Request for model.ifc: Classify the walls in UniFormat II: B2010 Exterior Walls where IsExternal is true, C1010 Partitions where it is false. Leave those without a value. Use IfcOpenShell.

First a look at what the model holds.

```python
import ifcopenshell
import ifcopenshell.util.element

model = ifcopenshell.open("model.ifc")
print(model.schema)
print("classifications:", [c.Name for c in model.by_type("IfcClassification")])
values = [ifcopenshell.util.element.get_pset(e, "Pset_WallCommon", "IsExternal") for e in model.by_type("IfcWall")]
for value in (True, False, None):
    print("IsExternal", value, values.count(value))
```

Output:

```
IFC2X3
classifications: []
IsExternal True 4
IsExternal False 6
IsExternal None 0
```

```python
import ifcopenshell
import ifcopenshell.api.classification
import ifcopenshell.util.element

model = ifcopenshell.open("model.ifc")

# IFC2X3 requires Source and Edition and has no link from the project to the system.
system = model.create_entity("IfcClassification", Source="ASTM", Edition="E1557", Name="UniFormat II")

walls = model.by_type("IfcWall")
external = {e: ifcopenshell.util.element.get_pset(e, "Pset_WallCommon", "IsExternal") for e in walls}
for flag, code, name in ((True, "B2010", "Exterior Walls"), (False, "C1010", "Partitions")):
    products = [e for e in walls if external[e] is flag]
    ifcopenshell.api.classification.add_reference(
        model, products=products, classification=system, identification=code, name=name
    )
    print(code, len(products))

model.write("model_rev.ifc")
```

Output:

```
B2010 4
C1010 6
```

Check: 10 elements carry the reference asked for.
